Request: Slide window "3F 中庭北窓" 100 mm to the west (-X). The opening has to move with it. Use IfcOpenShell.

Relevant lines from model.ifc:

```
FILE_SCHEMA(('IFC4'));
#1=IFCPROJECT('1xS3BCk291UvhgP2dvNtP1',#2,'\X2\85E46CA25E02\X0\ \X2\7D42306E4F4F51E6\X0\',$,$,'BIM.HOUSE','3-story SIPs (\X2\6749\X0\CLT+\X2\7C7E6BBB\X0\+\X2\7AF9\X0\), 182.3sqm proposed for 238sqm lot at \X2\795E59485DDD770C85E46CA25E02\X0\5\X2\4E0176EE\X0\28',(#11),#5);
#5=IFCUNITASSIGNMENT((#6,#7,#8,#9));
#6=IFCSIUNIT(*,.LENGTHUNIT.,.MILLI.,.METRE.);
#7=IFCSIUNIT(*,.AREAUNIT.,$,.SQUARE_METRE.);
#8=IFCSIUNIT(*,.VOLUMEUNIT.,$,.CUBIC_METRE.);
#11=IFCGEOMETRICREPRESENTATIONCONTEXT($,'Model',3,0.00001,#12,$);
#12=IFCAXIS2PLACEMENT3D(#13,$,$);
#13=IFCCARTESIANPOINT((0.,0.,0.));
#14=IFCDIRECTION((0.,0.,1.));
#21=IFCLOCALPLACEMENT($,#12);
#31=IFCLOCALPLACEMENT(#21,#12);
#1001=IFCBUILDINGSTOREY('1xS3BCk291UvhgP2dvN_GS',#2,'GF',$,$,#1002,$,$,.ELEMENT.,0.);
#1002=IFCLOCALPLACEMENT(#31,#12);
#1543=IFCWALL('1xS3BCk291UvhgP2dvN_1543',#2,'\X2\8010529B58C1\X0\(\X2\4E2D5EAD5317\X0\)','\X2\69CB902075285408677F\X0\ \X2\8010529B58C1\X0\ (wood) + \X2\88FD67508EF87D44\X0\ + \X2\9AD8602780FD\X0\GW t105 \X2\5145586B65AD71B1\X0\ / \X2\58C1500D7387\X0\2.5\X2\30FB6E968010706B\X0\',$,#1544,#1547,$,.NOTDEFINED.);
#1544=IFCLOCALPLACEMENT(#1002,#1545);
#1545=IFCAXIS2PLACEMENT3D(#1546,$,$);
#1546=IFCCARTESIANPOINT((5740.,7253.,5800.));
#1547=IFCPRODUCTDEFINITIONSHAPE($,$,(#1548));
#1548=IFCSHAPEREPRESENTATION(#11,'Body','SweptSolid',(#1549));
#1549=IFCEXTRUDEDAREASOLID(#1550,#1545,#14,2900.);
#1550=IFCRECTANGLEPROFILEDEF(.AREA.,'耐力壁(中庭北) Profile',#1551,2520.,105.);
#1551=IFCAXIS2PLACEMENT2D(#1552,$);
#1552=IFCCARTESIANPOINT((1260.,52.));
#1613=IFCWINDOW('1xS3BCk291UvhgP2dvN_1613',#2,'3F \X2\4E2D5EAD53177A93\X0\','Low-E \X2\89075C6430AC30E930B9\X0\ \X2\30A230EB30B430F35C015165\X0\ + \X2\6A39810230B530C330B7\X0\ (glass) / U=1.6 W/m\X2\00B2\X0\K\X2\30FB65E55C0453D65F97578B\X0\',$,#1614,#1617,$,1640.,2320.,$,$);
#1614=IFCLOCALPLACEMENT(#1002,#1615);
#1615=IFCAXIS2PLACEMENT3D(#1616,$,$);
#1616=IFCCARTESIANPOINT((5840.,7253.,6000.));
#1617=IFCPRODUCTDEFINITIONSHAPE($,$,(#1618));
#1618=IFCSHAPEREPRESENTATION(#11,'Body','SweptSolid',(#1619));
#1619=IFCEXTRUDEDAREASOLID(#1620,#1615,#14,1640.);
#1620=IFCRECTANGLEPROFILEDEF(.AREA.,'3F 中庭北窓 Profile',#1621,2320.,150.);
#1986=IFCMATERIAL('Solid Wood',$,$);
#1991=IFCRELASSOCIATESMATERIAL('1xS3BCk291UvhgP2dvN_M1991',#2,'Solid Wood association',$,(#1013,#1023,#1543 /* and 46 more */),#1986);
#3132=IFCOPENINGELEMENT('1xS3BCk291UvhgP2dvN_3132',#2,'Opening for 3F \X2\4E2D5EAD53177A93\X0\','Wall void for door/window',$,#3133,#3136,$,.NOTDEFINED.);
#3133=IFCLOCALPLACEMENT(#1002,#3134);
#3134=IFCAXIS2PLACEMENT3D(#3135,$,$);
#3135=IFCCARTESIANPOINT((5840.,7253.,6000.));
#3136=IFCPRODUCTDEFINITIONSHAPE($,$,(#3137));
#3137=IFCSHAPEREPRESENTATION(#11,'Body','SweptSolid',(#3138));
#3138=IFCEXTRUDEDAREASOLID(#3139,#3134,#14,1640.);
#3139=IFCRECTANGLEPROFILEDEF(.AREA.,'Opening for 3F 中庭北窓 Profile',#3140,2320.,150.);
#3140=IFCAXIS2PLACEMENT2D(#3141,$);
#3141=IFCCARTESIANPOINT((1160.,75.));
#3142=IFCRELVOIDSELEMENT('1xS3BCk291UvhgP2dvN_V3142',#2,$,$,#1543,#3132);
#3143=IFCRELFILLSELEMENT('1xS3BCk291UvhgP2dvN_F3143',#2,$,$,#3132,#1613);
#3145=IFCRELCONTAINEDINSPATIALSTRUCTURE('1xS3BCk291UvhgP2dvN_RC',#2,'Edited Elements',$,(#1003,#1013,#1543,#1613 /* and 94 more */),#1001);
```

```python
import ifcopenshell
import ifcopenshell.api.geometry
import ifcopenshell.util.placement

model = ifcopenshell.open("model.ifc")

window = model.by_guid("1xS3BCk291UvhgP2dvN_1613")
opening = window.FillsVoids[0].RelatingOpeningElement
wall = opening.VoidsElements[0].RelatingBuildingElement

wall_matrix = ifcopenshell.util.placement.get_local_placement(wall.ObjectPlacement)
shift = wall_matrix[:3, 0] * -100.0
before = ifcopenshell.util.placement.get_local_placement(window.ObjectPlacement)[:3, 3].copy()

# The window is not placed relative to its opening, so move both.
for product in (opening, window):
    matrix = ifcopenshell.util.placement.get_local_placement(product.ObjectPlacement)
    matrix[:3, 3] += shift
    ifcopenshell.api.geometry.edit_object_placement(model, product=product, matrix=matrix, is_si=False)

after = ifcopenshell.util.placement.get_local_placement(window.ObjectPlacement)[:3, 3]
print("window moved by", (after - before).round(3) + 0.0)

model.write("model_rev.ifc")
```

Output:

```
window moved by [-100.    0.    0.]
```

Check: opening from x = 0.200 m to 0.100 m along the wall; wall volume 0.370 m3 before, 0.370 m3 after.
